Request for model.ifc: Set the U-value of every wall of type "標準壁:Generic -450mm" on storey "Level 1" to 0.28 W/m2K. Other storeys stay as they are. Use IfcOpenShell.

First a look at what the model holds.

```python
import ifcopenshell
import ifcopenshell.util.element

model = ifcopenshell.open("model.ifc")
print(model.schema)
storey = next(s for s in model.by_type("IfcBuildingStorey") if s.Name == "Level 1")
walls = [e for e in ifcopenshell.util.element.get_decomposition(storey) if e.is_a("IfcWall")]
seen = {}
for e in walls:
    element_type = ifcopenshell.util.element.get_type(e)
    key = (element_type.Name if element_type != e and element_type else None, ifcopenshell.util.element.get_pset(e, "Pset_WallCommon", "ThermalTransmittance"))
    seen[key] = seen.get(key, 0) + 1
for (name, value), count in sorted(seen.items(), key=str):
    print(count, "x", name, "|", value)
```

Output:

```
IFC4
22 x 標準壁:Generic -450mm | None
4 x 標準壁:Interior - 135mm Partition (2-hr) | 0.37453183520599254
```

```python
import ifcopenshell
import ifcopenshell.api.pset
import ifcopenshell.util.element

model = ifcopenshell.open("model.ifc")

storey = next(s for s in model.by_type("IfcBuildingStorey") if s.Name == "Level 1")
walls = [e for e in ifcopenshell.util.element.get_decomposition(storey) if e.is_a("IfcWall")]

count = 0
for e in walls:
    element_type = ifcopenshell.util.element.get_type(e)
    if element_type in (None, e) or element_type.Name != "標準壁:Generic -450mm":
        continue
    # add_pset returns the element's existing set when there is one.
    pset = ifcopenshell.api.pset.add_pset(model, product=e, name="Pset_WallCommon")
    ifcopenshell.api.pset.edit_pset(model, pset=pset, properties={"ThermalTransmittance": 0.28})
    count += 1

print(count, "walls updated")

model.write("model_v2.ifc")
```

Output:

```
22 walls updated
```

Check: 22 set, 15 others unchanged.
